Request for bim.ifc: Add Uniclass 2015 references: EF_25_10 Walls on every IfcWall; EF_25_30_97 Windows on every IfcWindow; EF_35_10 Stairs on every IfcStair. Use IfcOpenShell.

First a look at what the model holds.

```python
import ifcopenshell

model = ifcopenshell.open("bim.ifc")
print(model.schema)
print("classifications:", [c.Name for c in model.by_type("IfcClassification")])
for ifc_class in ("IfcDoor", "IfcRoof", "IfcStair", "IfcWall", "IfcWindow"):
    print(ifc_class, len(model.by_type(ifc_class)))
```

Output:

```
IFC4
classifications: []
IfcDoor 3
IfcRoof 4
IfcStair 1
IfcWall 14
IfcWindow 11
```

```python
import ifcopenshell
import ifcopenshell.api.classification

model = ifcopenshell.open("bim.ifc")

system = ifcopenshell.api.classification.add_classification(model, classification="Uniclass 2015")

codes = {
    "IfcWall": ("EF_25_10", "Walls"),
    "IfcWindow": ("EF_25_30_97", "Windows"),
    "IfcStair": ("EF_35_10", "Stairs"),
}
for ifc_class, (code, name) in codes.items():
    products = model.by_type(ifc_class)
    ifcopenshell.api.classification.add_reference(
        model, products=products, classification=system, identification=code, name=name
    )
    print(code, len(products))

model.write("bim_updated.ifc")
```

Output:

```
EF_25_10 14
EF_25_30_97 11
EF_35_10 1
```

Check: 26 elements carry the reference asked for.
